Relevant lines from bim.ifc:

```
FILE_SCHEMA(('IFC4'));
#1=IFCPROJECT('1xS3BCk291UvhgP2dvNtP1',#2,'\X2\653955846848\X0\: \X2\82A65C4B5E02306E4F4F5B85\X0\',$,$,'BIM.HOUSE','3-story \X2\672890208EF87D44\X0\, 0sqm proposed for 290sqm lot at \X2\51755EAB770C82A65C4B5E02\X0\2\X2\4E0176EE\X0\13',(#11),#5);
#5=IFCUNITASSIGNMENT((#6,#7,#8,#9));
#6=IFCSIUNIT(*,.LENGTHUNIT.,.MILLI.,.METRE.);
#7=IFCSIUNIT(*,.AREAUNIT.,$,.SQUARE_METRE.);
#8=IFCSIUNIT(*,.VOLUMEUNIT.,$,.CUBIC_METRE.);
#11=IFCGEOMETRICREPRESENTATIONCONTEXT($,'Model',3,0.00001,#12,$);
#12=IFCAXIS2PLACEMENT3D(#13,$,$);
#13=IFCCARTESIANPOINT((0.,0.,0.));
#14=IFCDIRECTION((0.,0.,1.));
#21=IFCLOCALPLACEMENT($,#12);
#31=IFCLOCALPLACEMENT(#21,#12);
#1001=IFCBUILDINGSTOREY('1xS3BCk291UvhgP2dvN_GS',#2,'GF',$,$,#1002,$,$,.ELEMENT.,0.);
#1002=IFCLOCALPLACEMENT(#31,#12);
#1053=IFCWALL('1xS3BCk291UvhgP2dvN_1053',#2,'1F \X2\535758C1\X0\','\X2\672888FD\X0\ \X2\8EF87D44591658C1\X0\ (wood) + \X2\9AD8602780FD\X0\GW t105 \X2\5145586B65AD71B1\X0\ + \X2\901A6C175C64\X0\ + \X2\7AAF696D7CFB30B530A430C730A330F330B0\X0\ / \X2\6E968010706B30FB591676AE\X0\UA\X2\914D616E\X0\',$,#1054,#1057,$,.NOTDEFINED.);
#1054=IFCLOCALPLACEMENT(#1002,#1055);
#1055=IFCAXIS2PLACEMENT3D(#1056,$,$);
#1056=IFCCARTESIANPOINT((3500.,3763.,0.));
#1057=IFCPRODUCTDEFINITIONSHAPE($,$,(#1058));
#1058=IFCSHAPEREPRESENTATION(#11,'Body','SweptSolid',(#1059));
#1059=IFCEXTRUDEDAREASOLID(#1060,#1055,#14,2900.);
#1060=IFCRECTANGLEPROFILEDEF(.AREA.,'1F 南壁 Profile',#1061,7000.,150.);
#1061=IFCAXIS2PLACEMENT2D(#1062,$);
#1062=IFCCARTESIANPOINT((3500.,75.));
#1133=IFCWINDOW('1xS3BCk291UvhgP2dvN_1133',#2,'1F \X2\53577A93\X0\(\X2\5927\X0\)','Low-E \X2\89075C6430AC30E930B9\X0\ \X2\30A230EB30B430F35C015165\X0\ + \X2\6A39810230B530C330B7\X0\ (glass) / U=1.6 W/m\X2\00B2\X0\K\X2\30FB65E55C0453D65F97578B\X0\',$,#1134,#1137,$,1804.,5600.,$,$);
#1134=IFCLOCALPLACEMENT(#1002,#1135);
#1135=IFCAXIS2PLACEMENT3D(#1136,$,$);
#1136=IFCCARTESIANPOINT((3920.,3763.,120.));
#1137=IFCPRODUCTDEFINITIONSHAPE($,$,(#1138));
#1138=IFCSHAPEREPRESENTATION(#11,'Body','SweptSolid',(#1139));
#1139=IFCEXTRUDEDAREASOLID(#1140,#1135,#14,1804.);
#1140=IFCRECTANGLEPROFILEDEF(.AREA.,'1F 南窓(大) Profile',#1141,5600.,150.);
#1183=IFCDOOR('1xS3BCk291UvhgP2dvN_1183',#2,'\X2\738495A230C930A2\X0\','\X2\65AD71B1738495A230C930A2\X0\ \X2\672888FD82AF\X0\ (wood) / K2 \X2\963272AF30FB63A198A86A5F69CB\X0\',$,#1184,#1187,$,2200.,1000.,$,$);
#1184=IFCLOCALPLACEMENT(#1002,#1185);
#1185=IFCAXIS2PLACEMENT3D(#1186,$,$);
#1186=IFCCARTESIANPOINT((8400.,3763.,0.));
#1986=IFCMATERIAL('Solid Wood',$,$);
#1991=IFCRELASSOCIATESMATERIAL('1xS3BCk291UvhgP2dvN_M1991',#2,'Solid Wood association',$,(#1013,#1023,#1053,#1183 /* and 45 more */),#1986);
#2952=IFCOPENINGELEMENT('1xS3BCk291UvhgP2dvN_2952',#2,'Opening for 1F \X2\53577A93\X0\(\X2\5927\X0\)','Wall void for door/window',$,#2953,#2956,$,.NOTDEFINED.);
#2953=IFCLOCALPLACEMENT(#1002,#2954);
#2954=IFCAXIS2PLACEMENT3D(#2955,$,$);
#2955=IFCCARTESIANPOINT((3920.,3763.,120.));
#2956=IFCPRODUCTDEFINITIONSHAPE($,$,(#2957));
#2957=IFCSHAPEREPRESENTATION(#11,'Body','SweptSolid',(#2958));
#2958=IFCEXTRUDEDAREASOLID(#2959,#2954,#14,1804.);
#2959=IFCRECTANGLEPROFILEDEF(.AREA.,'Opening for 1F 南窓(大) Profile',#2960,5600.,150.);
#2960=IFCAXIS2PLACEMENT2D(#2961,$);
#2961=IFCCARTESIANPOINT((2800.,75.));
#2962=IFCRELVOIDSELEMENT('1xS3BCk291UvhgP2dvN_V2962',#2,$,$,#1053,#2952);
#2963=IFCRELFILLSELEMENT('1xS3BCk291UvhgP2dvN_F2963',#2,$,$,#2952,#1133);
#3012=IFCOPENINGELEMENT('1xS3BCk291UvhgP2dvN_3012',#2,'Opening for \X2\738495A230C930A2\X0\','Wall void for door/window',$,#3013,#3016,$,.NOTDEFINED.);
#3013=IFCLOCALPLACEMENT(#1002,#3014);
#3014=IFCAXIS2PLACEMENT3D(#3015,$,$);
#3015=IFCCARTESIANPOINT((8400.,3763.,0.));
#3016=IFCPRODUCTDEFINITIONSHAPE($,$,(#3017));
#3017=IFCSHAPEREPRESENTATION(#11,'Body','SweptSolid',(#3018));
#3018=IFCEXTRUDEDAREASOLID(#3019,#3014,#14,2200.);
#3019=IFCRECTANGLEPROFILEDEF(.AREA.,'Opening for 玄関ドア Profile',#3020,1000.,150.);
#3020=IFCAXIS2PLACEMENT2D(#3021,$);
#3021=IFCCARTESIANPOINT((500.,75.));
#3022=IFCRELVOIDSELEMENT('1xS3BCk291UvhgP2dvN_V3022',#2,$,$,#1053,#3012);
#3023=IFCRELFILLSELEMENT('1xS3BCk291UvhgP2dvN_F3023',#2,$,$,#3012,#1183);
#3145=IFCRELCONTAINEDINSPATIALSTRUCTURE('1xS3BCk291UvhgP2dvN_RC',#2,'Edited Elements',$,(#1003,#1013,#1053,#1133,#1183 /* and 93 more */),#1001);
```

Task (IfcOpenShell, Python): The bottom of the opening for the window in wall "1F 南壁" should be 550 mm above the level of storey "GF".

```python
import numpy as np
import ifcopenshell
import ifcopenshell.api.geometry
import ifcopenshell.geom
import ifcopenshell.util.element
import ifcopenshell.util.placement
import ifcopenshell.util.shape
import ifcopenshell.util.unit

model = ifcopenshell.open("bim.ifc")
unit_scale = ifcopenshell.util.unit.calculate_unit_scale(model)

window = model.by_guid("1xS3BCk291UvhgP2dvN_1133")
opening = window.FillsVoids[0].RelatingOpeningElement
storey = ifcopenshell.util.element.get_container(window, ifc_class="IfcBuildingStorey")
level = ifcopenshell.util.placement.get_local_placement(storey.ObjectPlacement)[2, 3]

# The opening's origin need not be at the sill, so measure its lowest point.
shape = ifcopenshell.geom.create_shape(ifcopenshell.geom.settings(), opening)
bottom = ifcopenshell.util.shape.get_shape_bottom_elevation(shape, shape.geometry) / unit_scale
dz = level + 550.0 - bottom

shift = np.array([0.0, 0.0, dz])
# The window is not placed relative to its opening, so move both.
for product in (opening, window):
    matrix = ifcopenshell.util.placement.get_local_placement(product.ObjectPlacement)
    matrix[:3, 3] += shift
    ifcopenshell.api.geometry.edit_object_placement(model, product=product, matrix=matrix, is_si=False)

print(f"moved by {dz * unit_scale:+.3f} m")

model.write("bim_updated.ifc")
```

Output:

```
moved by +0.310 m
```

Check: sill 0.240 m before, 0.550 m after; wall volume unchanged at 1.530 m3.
